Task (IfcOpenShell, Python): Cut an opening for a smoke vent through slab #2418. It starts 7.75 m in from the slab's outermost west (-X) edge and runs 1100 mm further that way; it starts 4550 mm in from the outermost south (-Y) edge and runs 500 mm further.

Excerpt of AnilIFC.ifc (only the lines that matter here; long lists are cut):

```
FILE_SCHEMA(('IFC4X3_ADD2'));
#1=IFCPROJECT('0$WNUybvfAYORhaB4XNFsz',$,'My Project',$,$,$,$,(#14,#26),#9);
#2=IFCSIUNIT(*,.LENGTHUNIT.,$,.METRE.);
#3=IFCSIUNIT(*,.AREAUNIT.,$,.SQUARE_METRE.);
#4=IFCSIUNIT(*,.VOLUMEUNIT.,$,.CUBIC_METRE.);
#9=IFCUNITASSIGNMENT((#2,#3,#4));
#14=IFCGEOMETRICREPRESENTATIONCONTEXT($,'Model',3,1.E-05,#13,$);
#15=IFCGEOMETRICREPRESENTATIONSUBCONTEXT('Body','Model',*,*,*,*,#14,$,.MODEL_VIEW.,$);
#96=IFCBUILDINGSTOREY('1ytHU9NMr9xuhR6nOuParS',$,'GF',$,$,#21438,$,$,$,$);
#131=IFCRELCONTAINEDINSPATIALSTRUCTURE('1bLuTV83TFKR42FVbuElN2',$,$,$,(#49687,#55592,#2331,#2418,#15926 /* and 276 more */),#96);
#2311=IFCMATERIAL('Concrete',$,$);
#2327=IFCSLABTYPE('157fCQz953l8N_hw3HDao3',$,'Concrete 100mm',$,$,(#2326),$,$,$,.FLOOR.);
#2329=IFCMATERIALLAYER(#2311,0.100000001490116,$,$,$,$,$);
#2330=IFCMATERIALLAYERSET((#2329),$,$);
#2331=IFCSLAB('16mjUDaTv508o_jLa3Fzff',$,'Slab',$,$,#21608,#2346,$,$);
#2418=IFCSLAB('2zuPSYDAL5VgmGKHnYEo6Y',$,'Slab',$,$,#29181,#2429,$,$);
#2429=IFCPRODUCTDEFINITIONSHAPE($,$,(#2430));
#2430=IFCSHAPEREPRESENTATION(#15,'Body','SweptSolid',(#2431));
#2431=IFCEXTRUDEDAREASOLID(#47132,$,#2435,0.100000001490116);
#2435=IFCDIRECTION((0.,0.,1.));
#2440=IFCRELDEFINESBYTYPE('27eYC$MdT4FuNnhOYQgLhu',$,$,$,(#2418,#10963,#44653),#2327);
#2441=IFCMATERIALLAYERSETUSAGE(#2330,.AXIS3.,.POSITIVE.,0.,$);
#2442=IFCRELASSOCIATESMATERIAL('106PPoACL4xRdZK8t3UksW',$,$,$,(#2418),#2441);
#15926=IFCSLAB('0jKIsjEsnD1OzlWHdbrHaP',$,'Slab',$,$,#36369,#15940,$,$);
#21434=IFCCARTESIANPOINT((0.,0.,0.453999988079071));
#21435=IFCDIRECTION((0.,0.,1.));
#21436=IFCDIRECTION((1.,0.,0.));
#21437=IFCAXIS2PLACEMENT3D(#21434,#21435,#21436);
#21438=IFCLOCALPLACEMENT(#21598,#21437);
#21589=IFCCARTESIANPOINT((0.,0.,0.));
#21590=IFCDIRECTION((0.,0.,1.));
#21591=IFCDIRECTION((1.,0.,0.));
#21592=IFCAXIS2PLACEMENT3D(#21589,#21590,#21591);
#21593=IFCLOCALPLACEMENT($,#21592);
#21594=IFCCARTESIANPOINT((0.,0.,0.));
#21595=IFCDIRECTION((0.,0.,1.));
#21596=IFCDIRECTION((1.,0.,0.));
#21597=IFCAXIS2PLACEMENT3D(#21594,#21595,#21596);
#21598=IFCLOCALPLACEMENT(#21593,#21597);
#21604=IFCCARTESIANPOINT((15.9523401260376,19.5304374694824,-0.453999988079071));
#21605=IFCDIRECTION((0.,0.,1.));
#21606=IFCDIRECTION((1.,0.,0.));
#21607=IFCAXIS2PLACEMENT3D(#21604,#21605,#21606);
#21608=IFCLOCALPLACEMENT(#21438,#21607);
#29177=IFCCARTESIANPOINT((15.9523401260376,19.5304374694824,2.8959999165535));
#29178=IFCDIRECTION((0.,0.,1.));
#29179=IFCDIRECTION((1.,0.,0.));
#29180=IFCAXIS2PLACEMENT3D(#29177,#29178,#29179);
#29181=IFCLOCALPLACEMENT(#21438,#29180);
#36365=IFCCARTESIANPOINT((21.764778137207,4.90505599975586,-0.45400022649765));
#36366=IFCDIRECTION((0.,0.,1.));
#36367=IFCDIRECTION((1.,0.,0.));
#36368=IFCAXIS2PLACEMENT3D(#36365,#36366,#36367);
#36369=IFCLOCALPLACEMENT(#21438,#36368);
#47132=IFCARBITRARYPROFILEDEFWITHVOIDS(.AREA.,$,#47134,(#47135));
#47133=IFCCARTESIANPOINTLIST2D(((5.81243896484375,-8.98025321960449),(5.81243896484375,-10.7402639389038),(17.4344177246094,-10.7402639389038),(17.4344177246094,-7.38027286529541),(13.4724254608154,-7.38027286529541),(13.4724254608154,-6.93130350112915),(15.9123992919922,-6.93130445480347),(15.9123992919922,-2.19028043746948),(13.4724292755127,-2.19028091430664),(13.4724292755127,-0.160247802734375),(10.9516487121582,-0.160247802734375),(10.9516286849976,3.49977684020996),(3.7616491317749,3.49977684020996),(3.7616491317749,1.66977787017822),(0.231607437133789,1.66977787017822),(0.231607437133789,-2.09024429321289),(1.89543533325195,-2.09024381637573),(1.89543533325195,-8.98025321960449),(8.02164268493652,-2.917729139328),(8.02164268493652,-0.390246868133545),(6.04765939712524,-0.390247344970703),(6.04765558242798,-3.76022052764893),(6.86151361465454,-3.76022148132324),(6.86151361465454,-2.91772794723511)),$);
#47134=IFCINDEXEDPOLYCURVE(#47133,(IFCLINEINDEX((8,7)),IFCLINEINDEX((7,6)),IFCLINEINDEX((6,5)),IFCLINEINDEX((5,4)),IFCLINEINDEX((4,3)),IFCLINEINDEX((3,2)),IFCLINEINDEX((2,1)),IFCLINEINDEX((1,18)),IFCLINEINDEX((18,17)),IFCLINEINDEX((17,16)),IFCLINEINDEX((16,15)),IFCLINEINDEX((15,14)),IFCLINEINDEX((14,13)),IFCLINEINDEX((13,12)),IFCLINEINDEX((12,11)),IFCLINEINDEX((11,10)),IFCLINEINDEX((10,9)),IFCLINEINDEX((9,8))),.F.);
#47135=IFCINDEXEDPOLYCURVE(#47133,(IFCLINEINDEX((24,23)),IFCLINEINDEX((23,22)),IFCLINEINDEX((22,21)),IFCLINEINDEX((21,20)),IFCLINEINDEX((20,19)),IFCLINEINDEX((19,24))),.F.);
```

```python
import numpy as np
import ifcopenshell
import ifcopenshell.api.feature
import ifcopenshell.api.geometry
import ifcopenshell.api.root
import ifcopenshell.geom
import ifcopenshell.util.placement
import ifcopenshell.util.representation
import ifcopenshell.util.shape
import ifcopenshell.util.unit

model = ifcopenshell.open("AnilIFC.ifc")
unit_scale = ifcopenshell.util.unit.calculate_unit_scale(model)
settings = ifcopenshell.geom.settings()


def volume(element):
    """Net volume in cubic metres, openings subtracted."""
    shape = ifcopenshell.geom.create_shape(settings, element)
    return ifcopenshell.util.shape.get_volume(shape.geometry)


slab = model.by_id(2418)
before = volume(slab)

# Extent in the slab's own axes, in metres. The edges named are its -X and -Y sides.
slab_shape = ifcopenshell.geom.create_shape(settings, slab)
vertices = ifcopenshell.util.shape.get_vertices(slab_shape.geometry)
x_min, y_min, bottom = vertices.min(axis=0)
top = vertices[:, 2].max()

opening = ifcopenshell.api.root.create_entity(model, ifc_class="IfcOpeningElement", name="Smoke vent opening", predefined_type="OPENING")
context = ifcopenshell.util.representation.get_context(model, "Model", "Body", "MODEL_VIEW")
width, depth = 1.1, 0.5
outline = [(0.0, 0.0), (width, 0.0), (width, depth), (0.0, depth), (0.0, 0.0)]
# Overshoot both faces by 50 mm so the cut is clean.
shape = ifcopenshell.api.geometry.add_slab_representation(
    model, context=context, depth=top - bottom + 0.1, polyline=outline
)
ifcopenshell.api.geometry.assign_representation(model, product=opening, representation=shape)

matrix = ifcopenshell.util.placement.get_local_placement(slab.ObjectPlacement)
matrix[:, 3] = matrix @ np.append(np.array([x_min + 7.75, y_min + 4.55, bottom - 0.05]) / unit_scale, 1.0)
ifcopenshell.api.geometry.edit_object_placement(model, product=opening, matrix=matrix, is_si=False)
ifcopenshell.api.feature.add_feature(model, feature=opening, element=slab)

after = volume(slab)

print(f"slab volume {before:.3f} -> {after:.3f} m3")

model.write("AnilIFC_v2.ifc")
```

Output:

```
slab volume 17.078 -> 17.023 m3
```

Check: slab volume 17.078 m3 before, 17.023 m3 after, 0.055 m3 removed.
